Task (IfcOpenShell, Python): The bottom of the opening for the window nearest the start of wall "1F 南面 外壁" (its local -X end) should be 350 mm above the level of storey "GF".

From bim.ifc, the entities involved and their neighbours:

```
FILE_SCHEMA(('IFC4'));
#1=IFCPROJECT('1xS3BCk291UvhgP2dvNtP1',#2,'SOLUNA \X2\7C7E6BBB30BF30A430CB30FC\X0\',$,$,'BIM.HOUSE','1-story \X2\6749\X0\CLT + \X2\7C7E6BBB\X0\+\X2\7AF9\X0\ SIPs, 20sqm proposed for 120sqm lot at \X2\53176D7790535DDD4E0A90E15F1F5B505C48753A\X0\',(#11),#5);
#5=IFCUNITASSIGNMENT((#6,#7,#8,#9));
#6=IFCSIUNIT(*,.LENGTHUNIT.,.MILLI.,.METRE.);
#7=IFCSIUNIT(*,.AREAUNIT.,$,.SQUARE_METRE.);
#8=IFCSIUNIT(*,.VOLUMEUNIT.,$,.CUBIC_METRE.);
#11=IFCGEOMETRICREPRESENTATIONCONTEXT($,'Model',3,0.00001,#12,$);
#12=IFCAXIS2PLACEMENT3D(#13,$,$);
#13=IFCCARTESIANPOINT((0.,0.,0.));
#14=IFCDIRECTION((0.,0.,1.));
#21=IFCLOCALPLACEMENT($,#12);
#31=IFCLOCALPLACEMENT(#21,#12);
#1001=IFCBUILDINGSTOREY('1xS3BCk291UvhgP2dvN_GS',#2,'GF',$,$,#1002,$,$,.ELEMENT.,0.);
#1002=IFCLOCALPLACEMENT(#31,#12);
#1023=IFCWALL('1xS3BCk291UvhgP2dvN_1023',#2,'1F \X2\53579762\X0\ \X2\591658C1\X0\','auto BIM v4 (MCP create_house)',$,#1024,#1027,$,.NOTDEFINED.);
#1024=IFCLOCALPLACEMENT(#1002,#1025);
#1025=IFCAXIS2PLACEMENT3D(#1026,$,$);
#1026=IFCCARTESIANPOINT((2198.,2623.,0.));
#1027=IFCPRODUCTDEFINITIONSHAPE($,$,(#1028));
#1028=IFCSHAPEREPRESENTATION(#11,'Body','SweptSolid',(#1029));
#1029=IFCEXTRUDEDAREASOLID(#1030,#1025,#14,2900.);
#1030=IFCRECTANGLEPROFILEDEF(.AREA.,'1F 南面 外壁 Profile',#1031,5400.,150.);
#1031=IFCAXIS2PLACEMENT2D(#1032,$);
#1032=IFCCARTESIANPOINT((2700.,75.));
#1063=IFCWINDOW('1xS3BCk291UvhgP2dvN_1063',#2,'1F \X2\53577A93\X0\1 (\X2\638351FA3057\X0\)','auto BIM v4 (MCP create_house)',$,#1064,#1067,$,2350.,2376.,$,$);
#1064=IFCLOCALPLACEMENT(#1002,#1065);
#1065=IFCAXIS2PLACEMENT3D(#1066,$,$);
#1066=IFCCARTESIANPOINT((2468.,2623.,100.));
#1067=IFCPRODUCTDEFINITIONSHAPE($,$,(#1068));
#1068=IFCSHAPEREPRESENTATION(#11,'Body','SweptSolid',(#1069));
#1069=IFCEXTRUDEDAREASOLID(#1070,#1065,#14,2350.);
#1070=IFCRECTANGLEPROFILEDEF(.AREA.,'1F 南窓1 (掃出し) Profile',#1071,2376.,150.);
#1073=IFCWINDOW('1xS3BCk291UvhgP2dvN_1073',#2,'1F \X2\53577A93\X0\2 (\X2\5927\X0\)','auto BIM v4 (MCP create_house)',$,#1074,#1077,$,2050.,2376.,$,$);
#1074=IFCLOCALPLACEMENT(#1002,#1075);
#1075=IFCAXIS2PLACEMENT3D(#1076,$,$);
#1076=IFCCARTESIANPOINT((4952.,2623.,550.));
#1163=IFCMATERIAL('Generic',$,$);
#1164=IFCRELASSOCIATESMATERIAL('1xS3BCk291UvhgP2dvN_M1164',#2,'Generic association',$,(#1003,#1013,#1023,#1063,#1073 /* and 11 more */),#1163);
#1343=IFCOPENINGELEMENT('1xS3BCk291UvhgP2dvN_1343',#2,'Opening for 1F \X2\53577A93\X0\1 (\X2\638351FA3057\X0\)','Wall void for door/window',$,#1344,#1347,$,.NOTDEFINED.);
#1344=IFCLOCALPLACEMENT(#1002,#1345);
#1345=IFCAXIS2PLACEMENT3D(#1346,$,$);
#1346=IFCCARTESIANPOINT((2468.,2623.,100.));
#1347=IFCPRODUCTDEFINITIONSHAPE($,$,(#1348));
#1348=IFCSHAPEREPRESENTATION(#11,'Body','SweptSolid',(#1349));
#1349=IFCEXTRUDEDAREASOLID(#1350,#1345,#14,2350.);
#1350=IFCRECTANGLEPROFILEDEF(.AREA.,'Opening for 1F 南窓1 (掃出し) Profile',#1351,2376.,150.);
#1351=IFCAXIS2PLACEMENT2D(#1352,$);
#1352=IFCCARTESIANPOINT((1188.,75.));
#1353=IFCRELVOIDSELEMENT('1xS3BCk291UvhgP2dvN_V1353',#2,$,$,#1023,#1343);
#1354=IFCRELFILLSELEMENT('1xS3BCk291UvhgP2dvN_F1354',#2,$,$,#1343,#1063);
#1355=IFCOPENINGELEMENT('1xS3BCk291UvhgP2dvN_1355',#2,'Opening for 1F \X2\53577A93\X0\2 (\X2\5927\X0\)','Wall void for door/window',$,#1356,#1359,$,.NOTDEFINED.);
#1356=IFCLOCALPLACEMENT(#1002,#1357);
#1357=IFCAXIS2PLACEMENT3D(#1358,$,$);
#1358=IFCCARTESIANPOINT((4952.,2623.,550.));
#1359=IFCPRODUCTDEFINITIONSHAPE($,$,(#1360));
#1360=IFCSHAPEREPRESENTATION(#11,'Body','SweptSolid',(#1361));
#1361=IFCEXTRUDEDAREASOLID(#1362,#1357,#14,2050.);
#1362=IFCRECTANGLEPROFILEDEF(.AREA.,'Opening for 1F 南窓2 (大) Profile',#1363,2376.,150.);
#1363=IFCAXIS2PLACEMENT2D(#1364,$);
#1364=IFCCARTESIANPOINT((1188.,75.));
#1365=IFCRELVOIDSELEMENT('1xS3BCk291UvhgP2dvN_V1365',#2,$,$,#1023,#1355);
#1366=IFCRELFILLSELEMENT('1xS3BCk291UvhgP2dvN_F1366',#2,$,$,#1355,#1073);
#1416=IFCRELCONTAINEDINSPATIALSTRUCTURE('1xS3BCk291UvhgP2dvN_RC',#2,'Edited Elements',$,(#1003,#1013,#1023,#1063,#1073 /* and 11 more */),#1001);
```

```python
import numpy as np
import ifcopenshell
import ifcopenshell.api.geometry
import ifcopenshell.geom
import ifcopenshell.util.element
import ifcopenshell.util.placement
import ifcopenshell.util.shape
import ifcopenshell.util.unit

model = ifcopenshell.open("bim.ifc")
unit_scale = ifcopenshell.util.unit.calculate_unit_scale(model)

window = model.by_guid("1xS3BCk291UvhgP2dvN_1063")
opening = window.FillsVoids[0].RelatingOpeningElement
storey = ifcopenshell.util.element.get_container(window, ifc_class="IfcBuildingStorey")
level = ifcopenshell.util.placement.get_local_placement(storey.ObjectPlacement)[2, 3]

# The opening's origin need not be at the sill, so measure its lowest point.
shape = ifcopenshell.geom.create_shape(ifcopenshell.geom.settings(), opening)
bottom = ifcopenshell.util.shape.get_shape_bottom_elevation(shape, shape.geometry) / unit_scale
dz = level + 350.0 - bottom

shift = np.array([0.0, 0.0, dz])
# The window is not placed relative to its opening, so move both.
for product in (opening, window):
    matrix = ifcopenshell.util.placement.get_local_placement(product.ObjectPlacement)
    matrix[:3, 3] += shift
    ifcopenshell.api.geometry.edit_object_placement(model, product=product, matrix=matrix, is_si=False)

print(f"moved by {dz * unit_scale:+.3f} m")

model.write("bim-out.ifc")
```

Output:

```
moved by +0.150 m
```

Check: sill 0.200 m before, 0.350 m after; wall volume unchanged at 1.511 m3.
